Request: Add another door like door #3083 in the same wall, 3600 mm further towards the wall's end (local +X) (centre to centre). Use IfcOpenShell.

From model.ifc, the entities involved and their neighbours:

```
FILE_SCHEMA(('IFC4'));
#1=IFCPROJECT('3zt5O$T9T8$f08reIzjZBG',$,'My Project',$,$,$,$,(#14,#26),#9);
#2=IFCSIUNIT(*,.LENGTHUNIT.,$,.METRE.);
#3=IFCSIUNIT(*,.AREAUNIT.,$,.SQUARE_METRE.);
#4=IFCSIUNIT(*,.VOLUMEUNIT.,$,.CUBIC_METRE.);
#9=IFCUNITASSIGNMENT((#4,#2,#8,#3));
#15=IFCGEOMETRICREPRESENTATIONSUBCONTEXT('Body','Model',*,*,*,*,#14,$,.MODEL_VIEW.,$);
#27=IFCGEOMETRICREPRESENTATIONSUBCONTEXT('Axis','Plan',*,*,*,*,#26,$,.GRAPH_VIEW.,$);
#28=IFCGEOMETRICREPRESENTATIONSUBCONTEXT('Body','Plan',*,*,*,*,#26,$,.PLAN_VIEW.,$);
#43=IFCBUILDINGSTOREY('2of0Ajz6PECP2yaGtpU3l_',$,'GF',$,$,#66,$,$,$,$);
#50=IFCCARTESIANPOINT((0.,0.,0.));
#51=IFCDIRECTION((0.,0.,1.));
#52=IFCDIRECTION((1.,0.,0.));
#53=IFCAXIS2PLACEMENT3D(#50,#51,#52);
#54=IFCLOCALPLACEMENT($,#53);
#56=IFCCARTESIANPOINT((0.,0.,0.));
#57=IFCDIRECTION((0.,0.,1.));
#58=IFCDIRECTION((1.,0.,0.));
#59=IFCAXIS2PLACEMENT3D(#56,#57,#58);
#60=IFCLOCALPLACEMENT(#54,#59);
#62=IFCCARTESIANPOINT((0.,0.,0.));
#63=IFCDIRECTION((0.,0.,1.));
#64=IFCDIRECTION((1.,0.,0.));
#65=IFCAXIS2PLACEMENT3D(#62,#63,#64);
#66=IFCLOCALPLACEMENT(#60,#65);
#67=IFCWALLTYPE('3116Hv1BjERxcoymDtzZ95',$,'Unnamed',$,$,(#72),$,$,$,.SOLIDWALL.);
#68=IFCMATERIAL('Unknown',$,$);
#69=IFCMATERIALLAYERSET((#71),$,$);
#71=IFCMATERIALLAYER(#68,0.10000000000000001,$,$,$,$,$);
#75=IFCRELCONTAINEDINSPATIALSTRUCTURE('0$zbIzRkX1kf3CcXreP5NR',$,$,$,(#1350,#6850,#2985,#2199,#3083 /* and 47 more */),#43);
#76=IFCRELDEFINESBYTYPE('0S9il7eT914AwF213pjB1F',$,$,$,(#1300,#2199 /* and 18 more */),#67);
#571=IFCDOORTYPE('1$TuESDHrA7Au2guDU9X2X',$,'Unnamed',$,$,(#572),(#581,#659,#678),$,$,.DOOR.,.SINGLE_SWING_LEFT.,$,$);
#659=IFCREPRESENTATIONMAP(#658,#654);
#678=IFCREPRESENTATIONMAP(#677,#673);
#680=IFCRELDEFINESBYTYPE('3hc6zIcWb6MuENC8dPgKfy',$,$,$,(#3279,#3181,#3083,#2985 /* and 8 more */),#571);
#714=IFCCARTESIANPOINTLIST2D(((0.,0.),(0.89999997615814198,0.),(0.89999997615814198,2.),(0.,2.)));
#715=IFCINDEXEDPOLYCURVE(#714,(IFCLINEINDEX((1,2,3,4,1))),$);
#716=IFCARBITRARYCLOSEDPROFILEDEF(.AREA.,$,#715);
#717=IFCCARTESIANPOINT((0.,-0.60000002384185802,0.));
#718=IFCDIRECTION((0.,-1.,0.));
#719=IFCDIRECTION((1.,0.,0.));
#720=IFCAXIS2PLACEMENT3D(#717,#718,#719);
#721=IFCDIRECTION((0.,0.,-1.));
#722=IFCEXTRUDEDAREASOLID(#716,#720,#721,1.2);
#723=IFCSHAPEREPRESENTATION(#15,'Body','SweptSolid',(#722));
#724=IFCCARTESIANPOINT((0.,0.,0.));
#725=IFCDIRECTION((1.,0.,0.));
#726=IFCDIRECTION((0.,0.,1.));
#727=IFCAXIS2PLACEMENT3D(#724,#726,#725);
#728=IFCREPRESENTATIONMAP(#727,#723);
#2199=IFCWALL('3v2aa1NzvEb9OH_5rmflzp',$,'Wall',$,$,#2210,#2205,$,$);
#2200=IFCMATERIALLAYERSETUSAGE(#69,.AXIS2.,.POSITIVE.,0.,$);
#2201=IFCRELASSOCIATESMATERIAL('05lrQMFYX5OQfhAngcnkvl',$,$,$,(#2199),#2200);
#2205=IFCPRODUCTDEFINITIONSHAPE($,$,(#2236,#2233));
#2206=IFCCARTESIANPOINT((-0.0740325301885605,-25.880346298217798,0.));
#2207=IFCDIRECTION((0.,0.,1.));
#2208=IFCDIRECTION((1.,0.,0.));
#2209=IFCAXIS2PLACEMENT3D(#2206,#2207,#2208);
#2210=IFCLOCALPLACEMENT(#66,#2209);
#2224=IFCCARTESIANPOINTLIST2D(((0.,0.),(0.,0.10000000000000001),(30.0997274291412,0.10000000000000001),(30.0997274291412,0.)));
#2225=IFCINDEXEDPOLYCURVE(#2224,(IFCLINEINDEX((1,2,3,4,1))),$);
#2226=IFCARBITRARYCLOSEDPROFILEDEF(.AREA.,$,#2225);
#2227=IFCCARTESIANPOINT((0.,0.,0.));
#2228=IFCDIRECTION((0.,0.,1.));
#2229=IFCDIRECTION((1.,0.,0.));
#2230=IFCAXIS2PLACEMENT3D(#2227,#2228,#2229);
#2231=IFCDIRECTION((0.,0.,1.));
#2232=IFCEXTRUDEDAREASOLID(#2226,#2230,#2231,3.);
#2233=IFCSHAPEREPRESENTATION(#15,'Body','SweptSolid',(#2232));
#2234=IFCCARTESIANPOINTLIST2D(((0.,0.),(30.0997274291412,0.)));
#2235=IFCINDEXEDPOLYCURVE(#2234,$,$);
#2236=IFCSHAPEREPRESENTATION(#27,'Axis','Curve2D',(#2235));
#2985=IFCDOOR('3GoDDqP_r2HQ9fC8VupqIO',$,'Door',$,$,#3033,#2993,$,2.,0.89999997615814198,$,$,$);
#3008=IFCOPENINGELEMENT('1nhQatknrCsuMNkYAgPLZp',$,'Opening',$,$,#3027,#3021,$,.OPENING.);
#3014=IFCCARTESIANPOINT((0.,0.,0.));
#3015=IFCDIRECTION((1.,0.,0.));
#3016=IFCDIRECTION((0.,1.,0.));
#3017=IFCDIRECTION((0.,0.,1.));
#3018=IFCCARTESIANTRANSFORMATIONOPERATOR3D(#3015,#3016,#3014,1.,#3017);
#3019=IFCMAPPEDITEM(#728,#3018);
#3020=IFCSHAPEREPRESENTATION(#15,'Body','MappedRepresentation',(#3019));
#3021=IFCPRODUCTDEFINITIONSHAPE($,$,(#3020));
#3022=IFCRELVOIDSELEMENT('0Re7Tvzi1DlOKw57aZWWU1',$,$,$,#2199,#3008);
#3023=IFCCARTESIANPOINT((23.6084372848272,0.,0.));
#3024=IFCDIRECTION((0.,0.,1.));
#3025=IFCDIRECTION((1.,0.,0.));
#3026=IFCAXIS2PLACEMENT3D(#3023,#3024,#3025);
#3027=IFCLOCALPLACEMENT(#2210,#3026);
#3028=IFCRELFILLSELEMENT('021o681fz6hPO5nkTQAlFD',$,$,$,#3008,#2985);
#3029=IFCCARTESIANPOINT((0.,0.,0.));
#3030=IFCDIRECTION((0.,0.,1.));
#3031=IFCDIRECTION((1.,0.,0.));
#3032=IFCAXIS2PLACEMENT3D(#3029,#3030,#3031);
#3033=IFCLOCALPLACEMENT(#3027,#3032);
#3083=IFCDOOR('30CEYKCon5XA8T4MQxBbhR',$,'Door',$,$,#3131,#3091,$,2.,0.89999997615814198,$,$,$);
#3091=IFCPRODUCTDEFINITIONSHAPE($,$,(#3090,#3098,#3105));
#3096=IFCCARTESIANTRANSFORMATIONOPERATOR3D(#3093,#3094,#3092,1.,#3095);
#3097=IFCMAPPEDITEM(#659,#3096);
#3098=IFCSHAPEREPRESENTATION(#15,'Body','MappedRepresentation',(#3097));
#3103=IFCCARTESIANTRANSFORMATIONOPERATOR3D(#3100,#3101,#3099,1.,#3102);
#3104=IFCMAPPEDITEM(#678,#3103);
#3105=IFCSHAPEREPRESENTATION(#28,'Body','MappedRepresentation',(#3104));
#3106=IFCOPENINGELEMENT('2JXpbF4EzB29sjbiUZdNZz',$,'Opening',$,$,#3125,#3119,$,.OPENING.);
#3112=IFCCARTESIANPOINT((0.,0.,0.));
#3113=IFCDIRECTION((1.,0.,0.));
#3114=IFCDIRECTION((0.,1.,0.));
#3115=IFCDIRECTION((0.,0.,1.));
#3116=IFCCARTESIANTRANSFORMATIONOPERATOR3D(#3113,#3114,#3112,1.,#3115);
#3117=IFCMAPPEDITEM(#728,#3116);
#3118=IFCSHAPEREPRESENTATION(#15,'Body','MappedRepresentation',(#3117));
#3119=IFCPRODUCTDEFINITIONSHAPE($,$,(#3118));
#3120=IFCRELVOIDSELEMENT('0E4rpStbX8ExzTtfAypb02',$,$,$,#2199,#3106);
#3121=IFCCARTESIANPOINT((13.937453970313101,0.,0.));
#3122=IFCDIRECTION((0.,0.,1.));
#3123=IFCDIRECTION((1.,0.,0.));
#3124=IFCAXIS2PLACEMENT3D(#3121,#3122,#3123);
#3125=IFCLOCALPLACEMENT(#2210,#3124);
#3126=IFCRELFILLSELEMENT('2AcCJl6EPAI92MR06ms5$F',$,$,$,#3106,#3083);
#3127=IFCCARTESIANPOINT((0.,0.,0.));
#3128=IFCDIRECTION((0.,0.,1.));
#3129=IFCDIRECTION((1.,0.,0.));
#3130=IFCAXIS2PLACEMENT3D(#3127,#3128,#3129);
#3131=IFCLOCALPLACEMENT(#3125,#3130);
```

```python
import ifcopenshell
import ifcopenshell.api.feature
import ifcopenshell.api.geometry
import ifcopenshell.api.root
import ifcopenshell.geom
import ifcopenshell.util.element
import ifcopenshell.util.placement
import ifcopenshell.util.shape
import ifcopenshell.util.unit

model = ifcopenshell.open("model.ifc")
unit_scale = ifcopenshell.util.unit.calculate_unit_scale(model)
settings = ifcopenshell.geom.settings()


def volume(element):
    """Net volume in cubic metres, openings subtracted."""
    shape = ifcopenshell.geom.create_shape(settings, element)
    return ifcopenshell.util.shape.get_volume(shape.geometry)


door = model.by_guid("30CEYKCon5XA8T4MQxBbhR")
opening = door.FillsVoids[0].RelatingOpeningElement
wall = opening.VoidsElements[0].RelatingBuildingElement
before = volume(wall)
shift = ifcopenshell.util.placement.get_local_placement(wall.ObjectPlacement)[:3, 0] * 3.6 / unit_scale

# copy_class copies the void relationship, type, container and properties, but no geometry.
new_opening = ifcopenshell.api.root.copy_class(model, product=opening)
new_opening.Representation = ifcopenshell.util.element.copy_deep(
    model, opening.Representation, exclude=["IfcGeometricRepresentationContext", "IfcRepresentationMap"]
)
new_door = ifcopenshell.api.root.copy_class(model, product=door)
new_door.Representation = ifcopenshell.util.element.copy_deep(
    model, door.Representation, exclude=["IfcGeometricRepresentationContext", "IfcRepresentationMap"]
)
ifcopenshell.api.feature.add_filling(model, opening=new_opening, element=new_door)

for old, new in ((opening, new_opening), (door, new_door)):
    matrix = ifcopenshell.util.placement.get_local_placement(old.ObjectPlacement)
    matrix[:3, 3] += shift
    ifcopenshell.api.geometry.edit_object_placement(model, product=new, matrix=matrix, is_si=False)

after = volume(wall)

print(f"wall volume {before:.3f} -> {after:.3f} m3")

model.write("model_v2.ifc")
```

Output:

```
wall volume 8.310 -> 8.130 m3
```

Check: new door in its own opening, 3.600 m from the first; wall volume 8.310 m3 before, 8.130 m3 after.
